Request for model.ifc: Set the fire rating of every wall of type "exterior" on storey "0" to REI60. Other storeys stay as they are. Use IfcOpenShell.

First a look at what the model holds.

```python
import ifcopenshell
import ifcopenshell.util.element

model = ifcopenshell.open("model.ifc")
print(model.schema)
storey = next(s for s in model.by_type("IfcBuildingStorey") if s.Name == "0")
walls = [e for e in ifcopenshell.util.element.get_decomposition(storey) if e.is_a("IfcWall")]
seen = {}
for e in walls:
    element_type = ifcopenshell.util.element.get_type(e)
    key = (element_type.Name if element_type != e and element_type else None, ifcopenshell.util.element.get_pset(e, "Pset_WallCommon", "FireRating"))
    seen[key] = seen.get(key, 0) + 1
for (name, value), count in sorted(seen.items(), key=str):
    print(count, "x", name, "|", value)
```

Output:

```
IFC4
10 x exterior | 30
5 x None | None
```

```python
import ifcopenshell
import ifcopenshell.api.pset
import ifcopenshell.util.element

model = ifcopenshell.open("model.ifc")

storey = next(s for s in model.by_type("IfcBuildingStorey") if s.Name == "0")
walls = [e for e in ifcopenshell.util.element.get_decomposition(storey) if e.is_a("IfcWall")]

count = 0
for e in walls:
    element_type = ifcopenshell.util.element.get_type(e)
    if element_type in (None, e) or element_type.Name != "exterior":
        continue
    # add_pset returns the element's existing set when there is one.
    pset = ifcopenshell.api.pset.add_pset(model, product=e, name="Pset_WallCommon")
    ifcopenshell.api.pset.edit_pset(model, pset=pset, properties={"FireRating": "REI60"})
    count += 1

print(count, "walls updated")

model.write("model_updated.ifc")
```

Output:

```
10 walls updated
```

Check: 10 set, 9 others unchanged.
